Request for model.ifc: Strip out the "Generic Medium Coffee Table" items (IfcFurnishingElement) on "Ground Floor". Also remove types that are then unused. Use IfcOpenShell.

First a look at what the model holds.

```python
import ifcopenshell
import ifcopenshell.util.element

model = ifcopenshell.open("model.ifc")
print(model.schema)
storey = next(s for s in model.by_type("IfcBuildingStorey") if s.Name == "Ground Floor")
furniture = [e for e in ifcopenshell.util.element.get_decomposition(storey) if e.is_a("IfcFurnishingElement")]
seen = {}
for e in furniture:
    element_type = ifcopenshell.util.element.get_type(e)
    name = element_type.Name if element_type not in (None, e) else None
    seen[name] = seen.get(name, 0) + 1
for name, count in sorted(seen.items(), key=str):
    print(count, "x", name)
```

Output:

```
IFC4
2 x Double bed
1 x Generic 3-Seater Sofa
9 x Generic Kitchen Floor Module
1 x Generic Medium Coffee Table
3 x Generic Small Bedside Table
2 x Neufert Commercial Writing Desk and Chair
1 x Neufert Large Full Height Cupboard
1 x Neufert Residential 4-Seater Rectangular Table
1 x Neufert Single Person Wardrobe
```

```python
import ifcopenshell
import ifcopenshell.api.root
import ifcopenshell.util.element

model = ifcopenshell.open("model.ifc")

storey = next(s for s in model.by_type("IfcBuildingStorey") if s.Name == "Ground Floor")
furniture = [e for e in ifcopenshell.util.element.get_decomposition(storey) if e.is_a("IfcFurnishingElement")]
targets = [e for e in furniture if (t := ifcopenshell.util.element.get_type(e)) not in (None, e) and t.Name == "Generic Medium Coffee Table"]
types = {ifcopenshell.util.element.get_type(e) for e in targets} - {None, *targets}

for e in targets:
    ifcopenshell.api.root.remove_product(model, product=e)
print(len(targets), "removed")

unused = [t for t in types if not ifcopenshell.util.element.get_types(t)]
for t in unused:
    ifcopenshell.api.root.remove_product(model, product=t)
print(len(unused), "unused types removed")

model.write("model-out.ifc")
```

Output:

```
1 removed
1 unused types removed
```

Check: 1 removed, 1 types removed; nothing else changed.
